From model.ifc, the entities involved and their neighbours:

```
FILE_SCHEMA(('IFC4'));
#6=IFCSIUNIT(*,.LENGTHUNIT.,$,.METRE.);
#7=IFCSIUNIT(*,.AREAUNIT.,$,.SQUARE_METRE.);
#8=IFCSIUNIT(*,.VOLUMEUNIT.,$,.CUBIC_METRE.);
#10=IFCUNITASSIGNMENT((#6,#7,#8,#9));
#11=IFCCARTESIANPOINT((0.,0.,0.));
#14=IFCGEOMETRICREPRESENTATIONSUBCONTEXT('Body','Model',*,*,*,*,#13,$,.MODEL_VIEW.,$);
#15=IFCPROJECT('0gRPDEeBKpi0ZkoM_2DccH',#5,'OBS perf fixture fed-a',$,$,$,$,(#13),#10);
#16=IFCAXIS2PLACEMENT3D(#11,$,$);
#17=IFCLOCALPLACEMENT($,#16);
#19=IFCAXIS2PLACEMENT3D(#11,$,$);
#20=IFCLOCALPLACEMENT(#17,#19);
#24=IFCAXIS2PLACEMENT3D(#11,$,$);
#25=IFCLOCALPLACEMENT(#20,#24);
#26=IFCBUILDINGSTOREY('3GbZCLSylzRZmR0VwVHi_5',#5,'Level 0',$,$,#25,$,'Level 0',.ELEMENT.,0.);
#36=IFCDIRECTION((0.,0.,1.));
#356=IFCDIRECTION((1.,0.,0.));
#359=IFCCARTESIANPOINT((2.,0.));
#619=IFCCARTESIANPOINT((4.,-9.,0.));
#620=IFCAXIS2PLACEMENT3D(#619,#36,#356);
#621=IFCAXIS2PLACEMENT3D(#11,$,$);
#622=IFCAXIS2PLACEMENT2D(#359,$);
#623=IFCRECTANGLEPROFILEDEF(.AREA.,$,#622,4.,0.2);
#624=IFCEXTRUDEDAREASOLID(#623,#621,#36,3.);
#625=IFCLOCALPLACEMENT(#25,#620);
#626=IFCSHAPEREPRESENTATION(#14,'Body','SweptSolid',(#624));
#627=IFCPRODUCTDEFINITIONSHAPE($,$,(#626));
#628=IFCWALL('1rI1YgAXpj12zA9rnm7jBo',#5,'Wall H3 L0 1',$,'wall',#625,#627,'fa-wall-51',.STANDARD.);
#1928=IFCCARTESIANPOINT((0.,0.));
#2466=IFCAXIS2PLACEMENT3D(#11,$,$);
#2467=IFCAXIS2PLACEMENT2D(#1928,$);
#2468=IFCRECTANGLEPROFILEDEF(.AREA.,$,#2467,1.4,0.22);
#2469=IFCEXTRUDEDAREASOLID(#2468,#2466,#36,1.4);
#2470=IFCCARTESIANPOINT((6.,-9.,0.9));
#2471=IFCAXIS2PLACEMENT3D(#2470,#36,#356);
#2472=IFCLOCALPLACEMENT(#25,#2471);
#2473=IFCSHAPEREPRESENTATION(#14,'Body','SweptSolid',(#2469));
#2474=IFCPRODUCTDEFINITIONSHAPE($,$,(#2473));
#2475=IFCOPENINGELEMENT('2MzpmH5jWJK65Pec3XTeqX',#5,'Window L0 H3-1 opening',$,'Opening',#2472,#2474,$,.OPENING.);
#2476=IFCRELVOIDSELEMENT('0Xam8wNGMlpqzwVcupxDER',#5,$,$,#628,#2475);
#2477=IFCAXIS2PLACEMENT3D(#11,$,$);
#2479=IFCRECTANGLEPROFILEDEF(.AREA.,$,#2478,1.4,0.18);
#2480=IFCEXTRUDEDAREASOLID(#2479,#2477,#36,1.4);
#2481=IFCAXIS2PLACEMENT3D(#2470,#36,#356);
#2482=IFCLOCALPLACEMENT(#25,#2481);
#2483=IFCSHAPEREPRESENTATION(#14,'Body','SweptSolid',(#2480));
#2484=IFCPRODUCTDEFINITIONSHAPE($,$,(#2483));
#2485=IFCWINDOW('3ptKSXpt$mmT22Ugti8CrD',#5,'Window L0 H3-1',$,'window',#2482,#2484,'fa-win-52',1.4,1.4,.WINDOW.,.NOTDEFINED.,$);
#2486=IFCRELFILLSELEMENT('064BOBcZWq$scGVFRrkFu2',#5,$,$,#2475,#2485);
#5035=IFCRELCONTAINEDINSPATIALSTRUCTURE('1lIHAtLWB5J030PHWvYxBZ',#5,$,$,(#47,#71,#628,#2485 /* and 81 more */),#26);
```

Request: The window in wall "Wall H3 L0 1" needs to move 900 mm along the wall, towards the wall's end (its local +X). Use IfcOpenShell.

```python
import ifcopenshell
import ifcopenshell.api.geometry
import ifcopenshell.util.placement

model = ifcopenshell.open("model.ifc")

window = model.by_guid("3ptKSXpt$mmT22Ugti8CrD")
opening = window.FillsVoids[0].RelatingOpeningElement
wall = opening.VoidsElements[0].RelatingBuildingElement

wall_matrix = ifcopenshell.util.placement.get_local_placement(wall.ObjectPlacement)
shift = wall_matrix[:3, 0] * 0.9
before = ifcopenshell.util.placement.get_local_placement(window.ObjectPlacement)[:3, 3].copy()

# The window is not placed relative to its opening, so move both.
for product in (opening, window):
    matrix = ifcopenshell.util.placement.get_local_placement(product.ObjectPlacement)
    matrix[:3, 3] += shift
    ifcopenshell.api.geometry.edit_object_placement(model, product=product, matrix=matrix, is_si=False)

after = ifcopenshell.util.placement.get_local_placement(window.ObjectPlacement)[:3, 3]
print("window moved by", (after - before).round(3) + 0.0)

model.write("model_updated.ifc")
```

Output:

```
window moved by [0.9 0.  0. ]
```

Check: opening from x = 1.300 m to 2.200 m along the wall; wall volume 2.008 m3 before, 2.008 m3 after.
